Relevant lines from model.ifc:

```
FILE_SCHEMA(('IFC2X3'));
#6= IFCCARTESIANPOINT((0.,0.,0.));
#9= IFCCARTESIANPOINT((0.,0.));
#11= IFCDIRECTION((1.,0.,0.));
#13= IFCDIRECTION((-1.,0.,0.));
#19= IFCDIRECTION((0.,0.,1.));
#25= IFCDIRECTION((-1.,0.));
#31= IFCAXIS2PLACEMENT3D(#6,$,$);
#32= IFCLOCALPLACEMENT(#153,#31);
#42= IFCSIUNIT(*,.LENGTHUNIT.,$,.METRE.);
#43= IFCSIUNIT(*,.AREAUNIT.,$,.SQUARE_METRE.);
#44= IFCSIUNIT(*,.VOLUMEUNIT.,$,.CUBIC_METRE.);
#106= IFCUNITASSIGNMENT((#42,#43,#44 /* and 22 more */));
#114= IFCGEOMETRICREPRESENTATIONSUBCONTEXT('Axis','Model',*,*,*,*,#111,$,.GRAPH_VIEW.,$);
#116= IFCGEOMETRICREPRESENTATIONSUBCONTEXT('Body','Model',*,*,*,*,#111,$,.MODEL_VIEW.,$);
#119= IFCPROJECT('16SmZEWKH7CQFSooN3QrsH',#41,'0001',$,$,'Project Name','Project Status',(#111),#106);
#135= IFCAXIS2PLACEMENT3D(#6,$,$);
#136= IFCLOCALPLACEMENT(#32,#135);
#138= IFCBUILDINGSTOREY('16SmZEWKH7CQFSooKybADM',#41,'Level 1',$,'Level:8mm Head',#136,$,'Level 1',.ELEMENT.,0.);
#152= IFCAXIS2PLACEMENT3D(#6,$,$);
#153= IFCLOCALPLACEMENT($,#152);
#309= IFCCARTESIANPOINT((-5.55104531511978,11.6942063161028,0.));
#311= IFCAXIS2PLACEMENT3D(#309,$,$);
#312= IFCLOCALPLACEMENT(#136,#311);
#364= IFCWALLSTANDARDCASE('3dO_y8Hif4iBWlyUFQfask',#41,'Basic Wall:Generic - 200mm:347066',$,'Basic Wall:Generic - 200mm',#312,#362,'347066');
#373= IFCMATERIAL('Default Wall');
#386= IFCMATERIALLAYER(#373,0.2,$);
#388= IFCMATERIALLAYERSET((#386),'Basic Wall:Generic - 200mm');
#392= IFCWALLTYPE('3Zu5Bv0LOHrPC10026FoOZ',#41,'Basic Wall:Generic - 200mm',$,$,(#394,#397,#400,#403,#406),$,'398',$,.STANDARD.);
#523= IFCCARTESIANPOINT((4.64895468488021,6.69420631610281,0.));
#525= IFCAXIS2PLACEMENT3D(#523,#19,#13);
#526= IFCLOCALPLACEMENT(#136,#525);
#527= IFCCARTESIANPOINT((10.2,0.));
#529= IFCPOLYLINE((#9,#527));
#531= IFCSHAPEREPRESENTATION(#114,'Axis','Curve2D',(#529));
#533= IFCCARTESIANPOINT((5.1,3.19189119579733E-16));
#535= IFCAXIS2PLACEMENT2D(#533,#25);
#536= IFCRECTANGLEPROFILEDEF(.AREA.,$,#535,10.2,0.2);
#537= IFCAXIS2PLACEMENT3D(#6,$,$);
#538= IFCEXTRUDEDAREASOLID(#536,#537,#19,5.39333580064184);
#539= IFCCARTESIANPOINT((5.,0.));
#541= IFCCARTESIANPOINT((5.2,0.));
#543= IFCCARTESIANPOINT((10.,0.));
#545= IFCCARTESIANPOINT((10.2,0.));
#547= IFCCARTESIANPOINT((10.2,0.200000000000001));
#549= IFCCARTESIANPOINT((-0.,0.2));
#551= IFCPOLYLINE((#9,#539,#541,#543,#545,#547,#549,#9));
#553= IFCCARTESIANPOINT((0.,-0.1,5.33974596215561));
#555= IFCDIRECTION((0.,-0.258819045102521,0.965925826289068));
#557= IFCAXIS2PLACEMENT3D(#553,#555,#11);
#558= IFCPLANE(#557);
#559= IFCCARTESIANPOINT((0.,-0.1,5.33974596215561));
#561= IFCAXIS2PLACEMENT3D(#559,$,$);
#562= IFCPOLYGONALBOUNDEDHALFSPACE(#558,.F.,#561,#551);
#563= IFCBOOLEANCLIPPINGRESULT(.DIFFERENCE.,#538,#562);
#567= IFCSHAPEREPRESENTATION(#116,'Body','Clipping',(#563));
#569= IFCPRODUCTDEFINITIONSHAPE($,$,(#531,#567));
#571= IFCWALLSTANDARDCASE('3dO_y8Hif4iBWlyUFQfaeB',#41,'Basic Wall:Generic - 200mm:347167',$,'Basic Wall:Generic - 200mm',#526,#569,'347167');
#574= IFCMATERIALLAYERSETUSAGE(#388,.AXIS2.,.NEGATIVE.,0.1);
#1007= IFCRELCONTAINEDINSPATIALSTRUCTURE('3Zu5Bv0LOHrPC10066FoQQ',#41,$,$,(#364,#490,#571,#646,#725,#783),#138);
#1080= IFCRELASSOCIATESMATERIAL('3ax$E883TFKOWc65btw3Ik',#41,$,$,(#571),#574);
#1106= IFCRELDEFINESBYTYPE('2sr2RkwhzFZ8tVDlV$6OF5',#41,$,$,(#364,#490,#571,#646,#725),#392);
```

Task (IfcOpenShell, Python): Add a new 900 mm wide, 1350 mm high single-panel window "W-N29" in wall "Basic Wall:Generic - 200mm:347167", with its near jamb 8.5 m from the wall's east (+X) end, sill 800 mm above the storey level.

```python
import numpy as np
import ifcopenshell
import ifcopenshell.api.feature
import ifcopenshell.api.geometry
import ifcopenshell.api.root
import ifcopenshell.api.spatial
import ifcopenshell.api.type
import ifcopenshell.geom
import ifcopenshell.util.element
import ifcopenshell.util.placement
import ifcopenshell.util.representation
import ifcopenshell.util.shape
import ifcopenshell.util.unit

model = ifcopenshell.open("model.ifc")
unit_scale = ifcopenshell.util.unit.calculate_unit_scale(model)
settings = ifcopenshell.geom.settings()


def volume(element):
    """Net volume in cubic metres, openings subtracted."""
    shape = ifcopenshell.geom.create_shape(settings, element)
    return ifcopenshell.util.shape.get_volume(shape.geometry)


wall = model.by_guid("3dO_y8Hif4iBWlyUFQfaeB")
storey = ifcopenshell.util.element.get_container(wall, ifc_class="IfcBuildingStorey")
context = ifcopenshell.util.representation.get_context(model, "Model", "Body", "MODEL_VIEW")
before = volume(wall)

width, height, from_end, sill = 0.9, 1.35, 8.5, 0.8  # metres

# The wall runs along its own X axis, and the end named is its -X end.
wall_shape = ifcopenshell.geom.create_shape(settings, wall)
x, y, z = ifcopenshell.util.shape.get_vertices(wall_shape.geometry).T
start = x.min() + from_end
face, thickness = float(y.min()), float(y.max() - y.min())
wall_matrix = ifcopenshell.util.placement.get_local_placement(wall.ObjectPlacement)
level = ifcopenshell.util.placement.get_local_placement(storey.ObjectPlacement)[2, 3]


def in_wall(x, y):
    """Placement at x, y metres in the wall's axes, at sill height."""
    matrix = wall_matrix.copy()
    matrix[:, 3] = wall_matrix @ np.array([x / unit_scale, y / unit_scale, 0.0, 1.0])
    matrix[2, 3] = level + sill / unit_scale
    return matrix


# Opening: a box that overshoots both wall faces by 50 mm.
opening = ifcopenshell.api.root.create_entity(model, ifc_class="IfcOpeningElement")
box = ifcopenshell.api.geometry.add_wall_representation(
    model, context=context, length=width, height=height, thickness=thickness + 0.1
)
ifcopenshell.api.geometry.assign_representation(model, product=opening, representation=box)
ifcopenshell.api.geometry.edit_object_placement(model, product=opening, matrix=in_wall(start, face - 0.05), is_si=False)
ifcopenshell.api.feature.add_feature(model, feature=opening, element=wall)

window = ifcopenshell.api.root.create_entity(model, ifc_class="IfcWindow", name="W-N29")
window.OverallWidth, window.OverallHeight = width / unit_scale, height / unit_scale
body = ifcopenshell.api.geometry.add_window_representation(
    model,
    context=context,
    overall_width=window.OverallWidth,
    overall_height=window.OverallHeight,
    partition_type="SINGLE_PANEL",
)
ifcopenshell.api.geometry.assign_representation(model, product=window, representation=body)
ifcopenshell.api.spatial.assign_container(model, products=[window], relating_structure=storey)
fills = ifcopenshell.api.feature.add_filling(model, opening=opening, element=window)
fills.OwnerHistory = window.OwnerHistory  # required in IFC2X3

# IFC2X3 keeps the operation on the window style.
style = ifcopenshell.api.root.create_entity(model, ifc_class="IfcWindowStyle", name="W-N29")
style.OperationType, style.ConstructionType = "SINGLE_PANEL", "NOTDEFINED"
style.ParameterTakesPrecedence = style.Sizeable = False
ifcopenshell.api.type.assign_type(model, related_objects=[window], relating_type=style)

# Centre the window in the wall's thickness.
ifcopenshell.api.geometry.edit_object_placement(model, product=window, matrix=in_wall(start, face), is_si=False)
window_shape = ifcopenshell.geom.create_shape(settings, window)
depth = ifcopenshell.util.shape.get_vertices(window_shape.geometry)[:, 1]
offset = face + thickness / 2 - (depth.min() + depth.max()) / 2
ifcopenshell.api.geometry.edit_object_placement(model, product=window, matrix=in_wall(start, offset), is_si=False)

after = volume(wall)

print(f"wall volume {before:.3f} -> {after:.3f} m3")

model.write("model_rev.ifc")
```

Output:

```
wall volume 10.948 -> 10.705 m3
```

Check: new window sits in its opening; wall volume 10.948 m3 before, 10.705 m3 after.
